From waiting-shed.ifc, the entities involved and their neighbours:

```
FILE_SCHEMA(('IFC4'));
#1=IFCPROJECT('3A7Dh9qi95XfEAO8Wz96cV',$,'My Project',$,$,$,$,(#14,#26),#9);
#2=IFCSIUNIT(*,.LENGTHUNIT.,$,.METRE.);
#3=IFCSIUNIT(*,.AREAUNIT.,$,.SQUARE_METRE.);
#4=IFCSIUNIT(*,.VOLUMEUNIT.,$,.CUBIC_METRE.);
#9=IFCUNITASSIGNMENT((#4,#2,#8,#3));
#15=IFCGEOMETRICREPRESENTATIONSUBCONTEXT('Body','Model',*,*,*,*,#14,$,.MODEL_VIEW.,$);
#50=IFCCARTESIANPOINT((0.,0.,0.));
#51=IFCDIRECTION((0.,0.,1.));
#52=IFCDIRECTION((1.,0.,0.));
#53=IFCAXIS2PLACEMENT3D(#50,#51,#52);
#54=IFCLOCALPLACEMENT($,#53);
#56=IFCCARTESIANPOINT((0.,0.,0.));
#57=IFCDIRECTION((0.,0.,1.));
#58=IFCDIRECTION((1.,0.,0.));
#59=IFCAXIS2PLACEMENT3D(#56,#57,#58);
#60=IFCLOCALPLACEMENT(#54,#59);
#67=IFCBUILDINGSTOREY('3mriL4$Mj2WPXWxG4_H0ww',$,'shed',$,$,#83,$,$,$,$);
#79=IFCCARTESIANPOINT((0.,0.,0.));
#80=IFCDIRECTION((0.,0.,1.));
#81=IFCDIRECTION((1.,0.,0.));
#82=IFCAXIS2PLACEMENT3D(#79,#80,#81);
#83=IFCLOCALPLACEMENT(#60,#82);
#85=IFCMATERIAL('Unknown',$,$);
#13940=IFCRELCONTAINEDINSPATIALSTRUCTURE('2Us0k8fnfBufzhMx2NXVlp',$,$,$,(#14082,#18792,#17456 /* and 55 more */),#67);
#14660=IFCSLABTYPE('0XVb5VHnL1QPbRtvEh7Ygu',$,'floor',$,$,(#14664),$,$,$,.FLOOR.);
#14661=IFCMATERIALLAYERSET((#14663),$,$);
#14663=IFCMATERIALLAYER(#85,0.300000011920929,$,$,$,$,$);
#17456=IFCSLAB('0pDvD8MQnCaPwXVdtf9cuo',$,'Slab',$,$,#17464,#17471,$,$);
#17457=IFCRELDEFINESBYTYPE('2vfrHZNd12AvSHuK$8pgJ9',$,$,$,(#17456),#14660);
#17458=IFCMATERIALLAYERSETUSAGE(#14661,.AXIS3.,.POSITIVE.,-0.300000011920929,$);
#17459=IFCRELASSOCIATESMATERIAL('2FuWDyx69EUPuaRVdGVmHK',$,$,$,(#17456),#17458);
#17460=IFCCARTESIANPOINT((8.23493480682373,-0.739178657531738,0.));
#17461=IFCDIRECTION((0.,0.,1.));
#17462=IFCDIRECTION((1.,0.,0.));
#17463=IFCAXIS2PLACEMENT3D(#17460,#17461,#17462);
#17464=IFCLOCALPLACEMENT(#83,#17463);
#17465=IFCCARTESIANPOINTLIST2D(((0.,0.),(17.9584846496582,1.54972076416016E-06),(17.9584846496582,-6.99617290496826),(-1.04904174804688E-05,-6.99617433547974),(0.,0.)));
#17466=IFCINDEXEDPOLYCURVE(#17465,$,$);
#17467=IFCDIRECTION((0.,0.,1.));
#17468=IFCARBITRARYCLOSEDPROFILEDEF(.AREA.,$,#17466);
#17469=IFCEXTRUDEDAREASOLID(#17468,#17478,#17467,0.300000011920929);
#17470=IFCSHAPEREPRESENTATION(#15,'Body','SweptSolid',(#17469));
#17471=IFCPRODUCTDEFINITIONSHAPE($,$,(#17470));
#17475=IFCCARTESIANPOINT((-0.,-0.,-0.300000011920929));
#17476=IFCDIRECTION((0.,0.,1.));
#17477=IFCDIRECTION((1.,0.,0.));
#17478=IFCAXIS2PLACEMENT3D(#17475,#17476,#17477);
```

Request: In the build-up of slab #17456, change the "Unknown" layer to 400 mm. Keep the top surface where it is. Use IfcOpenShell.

```python
import ifcopenshell
import ifcopenshell.util.element
import ifcopenshell.util.representation

model = ifcopenshell.open("waiting-shed.ifc")

layer_set = model.by_id(14661)
layer = next(l for l in layer_set.MaterialLayers if l.Material and l.Material.Name == "Unknown")
change = 0.4 - layer.LayerThickness
layer.LayerThickness += change

# Geometry does not follow the layer set by itself.
slabs = [e for e in ifcopenshell.util.element.get_elements_by_material(model, layer_set) if e.is_a("IfcSlab")]
for slab in sorted(slabs, key=lambda e: e.id()):
    body = ifcopenshell.util.representation.get_representation(slab, "Model", "Body")
    solid = body.Items[0]
    old_depth = solid.Depth
    solid.Depth += change
    # Extruded upwards: lower the start of the extrusion so the top stays.
    x, y, z = solid.Position.Location.Coordinates
    solid.Position.Location = model.createIfcCartesianPoint((x, y, z - change))
    print(slab.id(), f"{old_depth:g} -> {solid.Depth:g}")

# The layers are counted up from the underside, which has moved.
for usage in {ifcopenshell.util.element.get_material(slab) for slab in slabs}:
    usage.OffsetFromReferenceLine -= change

model.write("waiting-shed_rev.ifc")
```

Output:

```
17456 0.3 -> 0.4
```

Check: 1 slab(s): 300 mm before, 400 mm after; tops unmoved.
